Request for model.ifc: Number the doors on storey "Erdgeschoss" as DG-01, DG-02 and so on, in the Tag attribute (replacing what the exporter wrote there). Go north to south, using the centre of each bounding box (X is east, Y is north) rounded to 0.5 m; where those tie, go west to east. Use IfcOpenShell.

First a look at what the model holds.

```python
import ifcopenshell
import ifcopenshell.util.element
import ifcopenshell.util.placement

model = ifcopenshell.open("model.ifc")
print(model.schema)
storey = next(s for s in model.by_type("IfcBuildingStorey") if s.Name == "Erdgeschoss")
doors = [e for e in ifcopenshell.util.element.get_decomposition(storey) if e.is_a("IfcDoor")]
for e in sorted(doors, key=lambda e: e.id()):
    origin = ifcopenshell.util.placement.get_local_placement(e.ObjectPlacement)[:3, 3]
    print(e.id(), e.Tag, e.Name, origin.round(2) + 0.0, sep=" | ")
```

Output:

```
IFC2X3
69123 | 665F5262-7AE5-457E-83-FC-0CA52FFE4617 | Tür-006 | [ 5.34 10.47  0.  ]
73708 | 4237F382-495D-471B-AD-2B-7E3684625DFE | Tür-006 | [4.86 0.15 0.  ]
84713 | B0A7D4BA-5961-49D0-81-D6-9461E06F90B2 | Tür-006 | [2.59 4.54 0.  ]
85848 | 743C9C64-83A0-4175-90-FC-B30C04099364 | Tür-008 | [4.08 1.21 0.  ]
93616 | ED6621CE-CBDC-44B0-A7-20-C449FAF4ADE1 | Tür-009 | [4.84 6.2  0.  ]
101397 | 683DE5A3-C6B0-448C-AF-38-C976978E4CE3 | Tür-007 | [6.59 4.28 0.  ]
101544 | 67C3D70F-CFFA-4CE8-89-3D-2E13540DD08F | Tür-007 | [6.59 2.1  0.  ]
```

```python
import ifcopenshell
import ifcopenshell.geom
import ifcopenshell.util.element
import ifcopenshell.util.shape

model = ifcopenshell.open("model.ifc")
settings = ifcopenshell.geom.settings()
settings.set("use-world-coords", True)


def centre(element):
    shape = ifcopenshell.geom.create_shape(settings, element)
    return ifcopenshell.util.shape.get_bbox_centroid(shape.geometry)


storey = next(s for s in model.by_type("IfcBuildingStorey") if s.Name == "Erdgeschoss")
doors = [e for e in ifcopenshell.util.element.get_decomposition(storey) if e.is_a("IfcDoor")]

# Insertion points can sit at a corner or the storey origin, so sort by the geometry (in metres).
centres = {e: centre(e) for e in doors}
doors.sort(key=lambda e: (-round(centres[e][1] / 0.5), centres[e][0]))

for i, e in enumerate(doors, start=1):
    number = f"DG-{i:02d}"
    e.Tag = number
    print(e.id(), number)

model.write("model_edited.ifc")
```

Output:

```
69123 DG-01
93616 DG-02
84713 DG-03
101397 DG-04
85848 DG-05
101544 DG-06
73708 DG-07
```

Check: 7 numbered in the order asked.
